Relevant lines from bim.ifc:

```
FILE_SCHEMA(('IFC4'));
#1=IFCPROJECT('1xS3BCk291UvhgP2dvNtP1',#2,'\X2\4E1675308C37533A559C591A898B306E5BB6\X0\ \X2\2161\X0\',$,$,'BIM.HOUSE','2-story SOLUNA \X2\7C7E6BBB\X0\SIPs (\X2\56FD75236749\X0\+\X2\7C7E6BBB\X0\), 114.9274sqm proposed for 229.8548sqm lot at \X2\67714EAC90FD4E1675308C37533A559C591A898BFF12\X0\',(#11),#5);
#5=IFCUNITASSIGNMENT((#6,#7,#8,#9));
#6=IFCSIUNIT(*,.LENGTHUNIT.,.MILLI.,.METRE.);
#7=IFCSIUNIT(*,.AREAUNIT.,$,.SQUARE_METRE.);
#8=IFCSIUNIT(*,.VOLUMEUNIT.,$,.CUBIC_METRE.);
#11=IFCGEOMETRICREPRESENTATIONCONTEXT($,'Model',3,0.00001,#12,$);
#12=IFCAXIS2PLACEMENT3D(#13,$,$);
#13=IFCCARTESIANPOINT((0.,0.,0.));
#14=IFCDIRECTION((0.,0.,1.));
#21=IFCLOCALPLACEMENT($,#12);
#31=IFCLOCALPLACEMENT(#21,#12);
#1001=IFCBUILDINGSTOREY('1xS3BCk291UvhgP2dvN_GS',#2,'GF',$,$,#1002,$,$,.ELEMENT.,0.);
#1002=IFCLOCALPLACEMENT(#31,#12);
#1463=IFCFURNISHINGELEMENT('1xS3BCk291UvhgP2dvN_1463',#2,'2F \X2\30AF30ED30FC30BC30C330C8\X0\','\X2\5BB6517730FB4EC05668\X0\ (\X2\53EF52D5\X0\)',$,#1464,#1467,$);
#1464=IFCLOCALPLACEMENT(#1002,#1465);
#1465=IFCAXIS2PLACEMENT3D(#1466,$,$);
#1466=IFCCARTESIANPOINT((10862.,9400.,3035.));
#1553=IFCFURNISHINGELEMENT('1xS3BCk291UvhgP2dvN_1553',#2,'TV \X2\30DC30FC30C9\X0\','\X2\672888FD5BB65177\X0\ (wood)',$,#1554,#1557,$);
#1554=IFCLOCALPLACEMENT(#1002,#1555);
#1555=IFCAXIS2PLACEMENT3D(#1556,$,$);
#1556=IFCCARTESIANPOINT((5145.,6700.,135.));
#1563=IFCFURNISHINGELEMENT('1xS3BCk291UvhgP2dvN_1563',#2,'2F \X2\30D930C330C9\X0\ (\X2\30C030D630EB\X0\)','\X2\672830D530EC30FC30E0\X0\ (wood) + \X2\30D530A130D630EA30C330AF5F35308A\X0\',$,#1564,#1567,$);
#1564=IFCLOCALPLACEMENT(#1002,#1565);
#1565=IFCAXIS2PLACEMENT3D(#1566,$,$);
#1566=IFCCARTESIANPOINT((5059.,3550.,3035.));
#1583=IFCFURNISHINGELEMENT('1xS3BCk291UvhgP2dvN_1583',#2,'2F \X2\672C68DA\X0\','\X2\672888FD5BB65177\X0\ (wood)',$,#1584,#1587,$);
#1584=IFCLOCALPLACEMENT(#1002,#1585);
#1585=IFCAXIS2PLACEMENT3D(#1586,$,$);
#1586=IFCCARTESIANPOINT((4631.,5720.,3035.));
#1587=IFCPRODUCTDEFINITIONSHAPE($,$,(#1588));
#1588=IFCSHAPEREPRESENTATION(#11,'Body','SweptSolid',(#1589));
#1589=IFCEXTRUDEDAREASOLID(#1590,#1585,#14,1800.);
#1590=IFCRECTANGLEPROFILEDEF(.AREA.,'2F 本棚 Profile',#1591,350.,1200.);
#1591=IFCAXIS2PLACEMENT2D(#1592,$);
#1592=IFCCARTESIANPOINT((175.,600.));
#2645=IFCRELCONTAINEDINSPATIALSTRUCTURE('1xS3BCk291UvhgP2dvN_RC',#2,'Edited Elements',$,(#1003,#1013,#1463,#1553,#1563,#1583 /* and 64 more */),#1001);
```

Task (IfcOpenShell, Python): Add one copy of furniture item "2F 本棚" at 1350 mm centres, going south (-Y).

```python
import numpy as np
import ifcopenshell
import ifcopenshell.api.geometry
import ifcopenshell.api.root
import ifcopenshell.util.element
import ifcopenshell.util.placement
import ifcopenshell.util.unit

model = ifcopenshell.open("bim.ifc")
unit_scale = ifcopenshell.util.unit.calculate_unit_scale(model)


def reuse_history(source, copy):
    """copy_class also copies each property set's owner history, people and application; keep the originals."""
    for rel in copy.IsDefinedBy:
        if rel.is_a("IfcRelDefinesByProperties") and (history := rel.RelatingPropertyDefinition.OwnerHistory):
            rel.RelatingPropertyDefinition.OwnerHistory = source.OwnerHistory
            ifcopenshell.util.element.remove_deep2(model, history)


source = model.by_guid("1xS3BCk291UvhgP2dvN_1583")
base = ifcopenshell.util.placement.get_local_placement(source.ObjectPlacement)
step = np.array([0.0, -1.0, 0.0]) * 1.35 / unit_scale

for i in range(1, 2):
    copy = ifcopenshell.api.root.copy_class(model, product=source)
    copy.Representation = ifcopenshell.util.element.copy_deep(
        model, source.Representation, exclude=["IfcGeometricRepresentationContext", "IfcRepresentationMap"]
    )
    reuse_history(source, copy)
    matrix = base.copy()
    matrix[:3, 3] += i * step
    print("added at", matrix[:3, 3].round(3) + 0.0)
    ifcopenshell.api.geometry.edit_object_placement(model, product=copy, matrix=matrix, is_si=False)

model.write("bim_rev.ifc")
```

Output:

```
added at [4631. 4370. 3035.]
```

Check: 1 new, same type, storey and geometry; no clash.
